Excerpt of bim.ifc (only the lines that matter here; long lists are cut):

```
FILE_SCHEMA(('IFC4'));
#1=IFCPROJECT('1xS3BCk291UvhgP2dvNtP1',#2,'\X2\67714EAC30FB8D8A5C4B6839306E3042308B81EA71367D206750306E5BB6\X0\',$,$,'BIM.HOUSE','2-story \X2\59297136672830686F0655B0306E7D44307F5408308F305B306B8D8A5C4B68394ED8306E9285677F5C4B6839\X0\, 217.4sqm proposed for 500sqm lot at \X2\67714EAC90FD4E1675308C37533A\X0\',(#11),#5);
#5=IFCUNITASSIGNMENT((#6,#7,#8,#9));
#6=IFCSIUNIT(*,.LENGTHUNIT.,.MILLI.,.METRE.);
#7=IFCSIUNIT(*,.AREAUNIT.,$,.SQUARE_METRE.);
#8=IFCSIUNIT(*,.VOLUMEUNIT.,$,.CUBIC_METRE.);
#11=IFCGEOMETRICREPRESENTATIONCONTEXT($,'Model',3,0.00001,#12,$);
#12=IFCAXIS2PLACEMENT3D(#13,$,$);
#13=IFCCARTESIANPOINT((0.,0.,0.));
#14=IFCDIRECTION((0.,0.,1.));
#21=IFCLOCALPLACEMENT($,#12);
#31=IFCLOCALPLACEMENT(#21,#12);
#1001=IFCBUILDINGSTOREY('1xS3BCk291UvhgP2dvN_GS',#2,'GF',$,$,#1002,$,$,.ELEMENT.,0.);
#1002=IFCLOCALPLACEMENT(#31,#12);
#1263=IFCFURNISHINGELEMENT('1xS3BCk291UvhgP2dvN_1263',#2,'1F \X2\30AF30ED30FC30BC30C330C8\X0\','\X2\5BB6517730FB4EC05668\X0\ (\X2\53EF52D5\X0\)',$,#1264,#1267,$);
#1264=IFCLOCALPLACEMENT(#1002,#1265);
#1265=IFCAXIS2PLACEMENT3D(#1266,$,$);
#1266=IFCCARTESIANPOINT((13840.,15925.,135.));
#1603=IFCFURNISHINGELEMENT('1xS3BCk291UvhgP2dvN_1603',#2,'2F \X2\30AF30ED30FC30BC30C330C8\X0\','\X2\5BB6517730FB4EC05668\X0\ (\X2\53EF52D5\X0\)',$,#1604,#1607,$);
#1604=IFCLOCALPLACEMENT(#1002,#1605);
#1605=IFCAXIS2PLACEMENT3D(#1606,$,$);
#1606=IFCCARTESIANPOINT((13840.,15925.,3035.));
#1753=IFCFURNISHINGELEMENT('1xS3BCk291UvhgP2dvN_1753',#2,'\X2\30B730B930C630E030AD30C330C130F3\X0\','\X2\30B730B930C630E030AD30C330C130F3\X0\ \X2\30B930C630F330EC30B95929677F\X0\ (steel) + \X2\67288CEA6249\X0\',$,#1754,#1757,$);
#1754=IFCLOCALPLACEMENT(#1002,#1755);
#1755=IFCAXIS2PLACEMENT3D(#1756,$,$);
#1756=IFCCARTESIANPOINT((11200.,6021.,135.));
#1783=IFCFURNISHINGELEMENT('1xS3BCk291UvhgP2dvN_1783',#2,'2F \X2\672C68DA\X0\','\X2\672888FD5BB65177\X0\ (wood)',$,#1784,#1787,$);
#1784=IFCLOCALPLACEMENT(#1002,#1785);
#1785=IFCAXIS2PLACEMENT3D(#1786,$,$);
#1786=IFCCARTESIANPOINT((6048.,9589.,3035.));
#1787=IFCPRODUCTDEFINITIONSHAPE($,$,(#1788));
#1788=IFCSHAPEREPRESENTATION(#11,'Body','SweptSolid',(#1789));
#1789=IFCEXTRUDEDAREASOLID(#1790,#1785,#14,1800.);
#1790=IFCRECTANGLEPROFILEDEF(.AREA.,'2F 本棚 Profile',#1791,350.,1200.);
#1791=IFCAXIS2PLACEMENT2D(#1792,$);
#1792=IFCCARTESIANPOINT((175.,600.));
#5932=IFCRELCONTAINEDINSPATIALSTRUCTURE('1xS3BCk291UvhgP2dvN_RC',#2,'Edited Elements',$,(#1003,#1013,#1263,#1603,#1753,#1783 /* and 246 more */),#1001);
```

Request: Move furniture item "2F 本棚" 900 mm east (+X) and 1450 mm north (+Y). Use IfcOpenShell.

```python
import ifcopenshell
import ifcopenshell.api.geometry
import ifcopenshell.util.placement

model = ifcopenshell.open("bim.ifc")

item = model.by_id(1783)
matrix = ifcopenshell.util.placement.get_local_placement(item.ObjectPlacement)
matrix[0, 3] += 900.0
matrix[1, 3] += 1450.0
ifcopenshell.api.geometry.edit_object_placement(model, product=item, matrix=matrix, is_si=False)

print(ifcopenshell.util.placement.get_local_placement(item.ObjectPlacement).round(3) + 0.0)

model.write("bim-out.ifc")
```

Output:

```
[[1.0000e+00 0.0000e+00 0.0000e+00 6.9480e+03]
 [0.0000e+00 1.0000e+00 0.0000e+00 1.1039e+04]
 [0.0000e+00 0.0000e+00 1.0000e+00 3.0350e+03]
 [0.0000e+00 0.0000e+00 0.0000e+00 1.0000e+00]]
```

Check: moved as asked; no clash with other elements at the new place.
